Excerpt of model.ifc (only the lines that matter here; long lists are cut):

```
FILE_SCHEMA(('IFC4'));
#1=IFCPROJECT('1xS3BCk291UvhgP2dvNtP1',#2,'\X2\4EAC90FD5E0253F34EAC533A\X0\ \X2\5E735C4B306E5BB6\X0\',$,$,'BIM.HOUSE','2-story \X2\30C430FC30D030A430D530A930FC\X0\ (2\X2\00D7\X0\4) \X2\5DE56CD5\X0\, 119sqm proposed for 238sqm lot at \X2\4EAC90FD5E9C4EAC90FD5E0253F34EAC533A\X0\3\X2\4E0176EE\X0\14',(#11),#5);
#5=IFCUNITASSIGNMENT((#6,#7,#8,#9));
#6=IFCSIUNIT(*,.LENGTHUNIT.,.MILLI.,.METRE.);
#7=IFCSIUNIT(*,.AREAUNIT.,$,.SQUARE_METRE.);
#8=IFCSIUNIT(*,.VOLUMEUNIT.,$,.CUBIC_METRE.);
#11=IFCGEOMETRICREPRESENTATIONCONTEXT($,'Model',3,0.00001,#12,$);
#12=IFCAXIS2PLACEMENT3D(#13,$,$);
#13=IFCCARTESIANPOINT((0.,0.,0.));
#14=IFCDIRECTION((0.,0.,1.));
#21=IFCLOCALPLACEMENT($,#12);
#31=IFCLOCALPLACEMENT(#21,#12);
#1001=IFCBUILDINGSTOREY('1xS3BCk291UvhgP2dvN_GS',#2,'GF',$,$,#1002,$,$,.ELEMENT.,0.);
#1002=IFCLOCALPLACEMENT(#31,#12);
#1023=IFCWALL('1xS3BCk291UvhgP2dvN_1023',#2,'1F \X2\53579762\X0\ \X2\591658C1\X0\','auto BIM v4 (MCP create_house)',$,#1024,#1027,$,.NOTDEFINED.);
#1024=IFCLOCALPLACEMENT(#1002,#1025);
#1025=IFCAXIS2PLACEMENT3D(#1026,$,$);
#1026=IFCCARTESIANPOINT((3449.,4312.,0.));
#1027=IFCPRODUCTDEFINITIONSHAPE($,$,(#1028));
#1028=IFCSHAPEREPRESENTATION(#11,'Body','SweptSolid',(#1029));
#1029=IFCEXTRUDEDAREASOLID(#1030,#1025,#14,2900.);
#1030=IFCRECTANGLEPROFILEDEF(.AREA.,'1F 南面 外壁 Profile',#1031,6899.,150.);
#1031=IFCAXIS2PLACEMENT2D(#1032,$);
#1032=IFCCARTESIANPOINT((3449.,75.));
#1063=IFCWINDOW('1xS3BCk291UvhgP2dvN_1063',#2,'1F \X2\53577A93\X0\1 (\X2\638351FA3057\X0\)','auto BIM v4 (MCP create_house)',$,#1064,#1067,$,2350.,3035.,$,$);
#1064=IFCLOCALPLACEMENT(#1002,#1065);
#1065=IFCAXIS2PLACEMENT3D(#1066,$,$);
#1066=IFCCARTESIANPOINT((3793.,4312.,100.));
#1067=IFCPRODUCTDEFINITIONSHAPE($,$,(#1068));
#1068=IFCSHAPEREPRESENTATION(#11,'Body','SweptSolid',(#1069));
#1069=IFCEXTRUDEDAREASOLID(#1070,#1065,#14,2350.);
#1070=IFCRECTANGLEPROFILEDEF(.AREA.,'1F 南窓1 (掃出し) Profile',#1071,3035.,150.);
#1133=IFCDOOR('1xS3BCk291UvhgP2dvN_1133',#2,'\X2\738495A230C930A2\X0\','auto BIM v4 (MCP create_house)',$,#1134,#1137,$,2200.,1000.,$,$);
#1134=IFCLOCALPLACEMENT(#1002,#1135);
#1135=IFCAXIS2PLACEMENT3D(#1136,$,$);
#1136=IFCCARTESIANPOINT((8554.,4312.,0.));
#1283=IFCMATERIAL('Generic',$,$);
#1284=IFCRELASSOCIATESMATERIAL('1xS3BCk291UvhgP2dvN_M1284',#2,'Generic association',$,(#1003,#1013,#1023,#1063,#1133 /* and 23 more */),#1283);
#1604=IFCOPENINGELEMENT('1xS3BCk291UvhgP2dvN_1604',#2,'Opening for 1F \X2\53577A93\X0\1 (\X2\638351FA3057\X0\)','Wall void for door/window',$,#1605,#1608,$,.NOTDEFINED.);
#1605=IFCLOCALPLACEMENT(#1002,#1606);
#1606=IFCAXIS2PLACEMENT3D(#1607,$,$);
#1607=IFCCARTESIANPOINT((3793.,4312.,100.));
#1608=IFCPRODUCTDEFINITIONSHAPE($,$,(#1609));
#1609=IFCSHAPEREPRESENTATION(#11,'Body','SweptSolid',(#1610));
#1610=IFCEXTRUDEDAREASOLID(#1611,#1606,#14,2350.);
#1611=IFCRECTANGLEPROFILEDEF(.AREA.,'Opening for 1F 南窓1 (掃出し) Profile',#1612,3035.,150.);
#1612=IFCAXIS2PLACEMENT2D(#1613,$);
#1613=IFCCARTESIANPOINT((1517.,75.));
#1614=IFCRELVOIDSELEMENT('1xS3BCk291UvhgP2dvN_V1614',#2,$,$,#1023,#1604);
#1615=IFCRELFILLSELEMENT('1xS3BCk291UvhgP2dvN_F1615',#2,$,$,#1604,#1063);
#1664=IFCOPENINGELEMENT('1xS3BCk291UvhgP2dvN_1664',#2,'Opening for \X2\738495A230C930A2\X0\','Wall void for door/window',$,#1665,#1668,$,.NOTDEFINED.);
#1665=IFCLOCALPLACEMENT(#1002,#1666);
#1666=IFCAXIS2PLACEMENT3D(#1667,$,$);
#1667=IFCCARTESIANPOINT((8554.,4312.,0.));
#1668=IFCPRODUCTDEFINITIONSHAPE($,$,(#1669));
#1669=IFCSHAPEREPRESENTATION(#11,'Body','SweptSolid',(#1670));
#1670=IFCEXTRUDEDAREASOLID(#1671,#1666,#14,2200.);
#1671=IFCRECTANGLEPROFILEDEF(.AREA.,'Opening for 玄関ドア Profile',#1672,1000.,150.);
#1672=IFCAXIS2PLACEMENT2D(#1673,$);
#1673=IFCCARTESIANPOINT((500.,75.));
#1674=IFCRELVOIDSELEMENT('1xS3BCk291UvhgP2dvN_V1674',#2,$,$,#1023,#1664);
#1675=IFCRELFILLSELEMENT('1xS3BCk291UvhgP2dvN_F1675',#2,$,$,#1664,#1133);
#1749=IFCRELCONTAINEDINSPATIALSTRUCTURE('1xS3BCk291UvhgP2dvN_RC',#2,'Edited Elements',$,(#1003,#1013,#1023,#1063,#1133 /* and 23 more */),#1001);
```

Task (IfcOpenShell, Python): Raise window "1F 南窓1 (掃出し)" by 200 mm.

```python
import numpy as np
import ifcopenshell
import ifcopenshell.api.geometry
import ifcopenshell.util.placement
import ifcopenshell.util.unit

model = ifcopenshell.open("model.ifc")
unit_scale = ifcopenshell.util.unit.calculate_unit_scale(model)

window = model.by_id(1063)
opening = window.FillsVoids[0].RelatingOpeningElement
dz = 0.2 / unit_scale

shift = np.array([0.0, 0.0, dz])
# The window is not placed relative to its opening, so move both.
for product in (opening, window):
    matrix = ifcopenshell.util.placement.get_local_placement(product.ObjectPlacement)
    matrix[:3, 3] += shift
    ifcopenshell.api.geometry.edit_object_placement(model, product=product, matrix=matrix, is_si=False)

print(f"moved by {dz * unit_scale:+.3f} m")

model.write("model_edited.ifc")
```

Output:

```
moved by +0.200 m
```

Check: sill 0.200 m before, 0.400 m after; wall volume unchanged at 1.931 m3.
